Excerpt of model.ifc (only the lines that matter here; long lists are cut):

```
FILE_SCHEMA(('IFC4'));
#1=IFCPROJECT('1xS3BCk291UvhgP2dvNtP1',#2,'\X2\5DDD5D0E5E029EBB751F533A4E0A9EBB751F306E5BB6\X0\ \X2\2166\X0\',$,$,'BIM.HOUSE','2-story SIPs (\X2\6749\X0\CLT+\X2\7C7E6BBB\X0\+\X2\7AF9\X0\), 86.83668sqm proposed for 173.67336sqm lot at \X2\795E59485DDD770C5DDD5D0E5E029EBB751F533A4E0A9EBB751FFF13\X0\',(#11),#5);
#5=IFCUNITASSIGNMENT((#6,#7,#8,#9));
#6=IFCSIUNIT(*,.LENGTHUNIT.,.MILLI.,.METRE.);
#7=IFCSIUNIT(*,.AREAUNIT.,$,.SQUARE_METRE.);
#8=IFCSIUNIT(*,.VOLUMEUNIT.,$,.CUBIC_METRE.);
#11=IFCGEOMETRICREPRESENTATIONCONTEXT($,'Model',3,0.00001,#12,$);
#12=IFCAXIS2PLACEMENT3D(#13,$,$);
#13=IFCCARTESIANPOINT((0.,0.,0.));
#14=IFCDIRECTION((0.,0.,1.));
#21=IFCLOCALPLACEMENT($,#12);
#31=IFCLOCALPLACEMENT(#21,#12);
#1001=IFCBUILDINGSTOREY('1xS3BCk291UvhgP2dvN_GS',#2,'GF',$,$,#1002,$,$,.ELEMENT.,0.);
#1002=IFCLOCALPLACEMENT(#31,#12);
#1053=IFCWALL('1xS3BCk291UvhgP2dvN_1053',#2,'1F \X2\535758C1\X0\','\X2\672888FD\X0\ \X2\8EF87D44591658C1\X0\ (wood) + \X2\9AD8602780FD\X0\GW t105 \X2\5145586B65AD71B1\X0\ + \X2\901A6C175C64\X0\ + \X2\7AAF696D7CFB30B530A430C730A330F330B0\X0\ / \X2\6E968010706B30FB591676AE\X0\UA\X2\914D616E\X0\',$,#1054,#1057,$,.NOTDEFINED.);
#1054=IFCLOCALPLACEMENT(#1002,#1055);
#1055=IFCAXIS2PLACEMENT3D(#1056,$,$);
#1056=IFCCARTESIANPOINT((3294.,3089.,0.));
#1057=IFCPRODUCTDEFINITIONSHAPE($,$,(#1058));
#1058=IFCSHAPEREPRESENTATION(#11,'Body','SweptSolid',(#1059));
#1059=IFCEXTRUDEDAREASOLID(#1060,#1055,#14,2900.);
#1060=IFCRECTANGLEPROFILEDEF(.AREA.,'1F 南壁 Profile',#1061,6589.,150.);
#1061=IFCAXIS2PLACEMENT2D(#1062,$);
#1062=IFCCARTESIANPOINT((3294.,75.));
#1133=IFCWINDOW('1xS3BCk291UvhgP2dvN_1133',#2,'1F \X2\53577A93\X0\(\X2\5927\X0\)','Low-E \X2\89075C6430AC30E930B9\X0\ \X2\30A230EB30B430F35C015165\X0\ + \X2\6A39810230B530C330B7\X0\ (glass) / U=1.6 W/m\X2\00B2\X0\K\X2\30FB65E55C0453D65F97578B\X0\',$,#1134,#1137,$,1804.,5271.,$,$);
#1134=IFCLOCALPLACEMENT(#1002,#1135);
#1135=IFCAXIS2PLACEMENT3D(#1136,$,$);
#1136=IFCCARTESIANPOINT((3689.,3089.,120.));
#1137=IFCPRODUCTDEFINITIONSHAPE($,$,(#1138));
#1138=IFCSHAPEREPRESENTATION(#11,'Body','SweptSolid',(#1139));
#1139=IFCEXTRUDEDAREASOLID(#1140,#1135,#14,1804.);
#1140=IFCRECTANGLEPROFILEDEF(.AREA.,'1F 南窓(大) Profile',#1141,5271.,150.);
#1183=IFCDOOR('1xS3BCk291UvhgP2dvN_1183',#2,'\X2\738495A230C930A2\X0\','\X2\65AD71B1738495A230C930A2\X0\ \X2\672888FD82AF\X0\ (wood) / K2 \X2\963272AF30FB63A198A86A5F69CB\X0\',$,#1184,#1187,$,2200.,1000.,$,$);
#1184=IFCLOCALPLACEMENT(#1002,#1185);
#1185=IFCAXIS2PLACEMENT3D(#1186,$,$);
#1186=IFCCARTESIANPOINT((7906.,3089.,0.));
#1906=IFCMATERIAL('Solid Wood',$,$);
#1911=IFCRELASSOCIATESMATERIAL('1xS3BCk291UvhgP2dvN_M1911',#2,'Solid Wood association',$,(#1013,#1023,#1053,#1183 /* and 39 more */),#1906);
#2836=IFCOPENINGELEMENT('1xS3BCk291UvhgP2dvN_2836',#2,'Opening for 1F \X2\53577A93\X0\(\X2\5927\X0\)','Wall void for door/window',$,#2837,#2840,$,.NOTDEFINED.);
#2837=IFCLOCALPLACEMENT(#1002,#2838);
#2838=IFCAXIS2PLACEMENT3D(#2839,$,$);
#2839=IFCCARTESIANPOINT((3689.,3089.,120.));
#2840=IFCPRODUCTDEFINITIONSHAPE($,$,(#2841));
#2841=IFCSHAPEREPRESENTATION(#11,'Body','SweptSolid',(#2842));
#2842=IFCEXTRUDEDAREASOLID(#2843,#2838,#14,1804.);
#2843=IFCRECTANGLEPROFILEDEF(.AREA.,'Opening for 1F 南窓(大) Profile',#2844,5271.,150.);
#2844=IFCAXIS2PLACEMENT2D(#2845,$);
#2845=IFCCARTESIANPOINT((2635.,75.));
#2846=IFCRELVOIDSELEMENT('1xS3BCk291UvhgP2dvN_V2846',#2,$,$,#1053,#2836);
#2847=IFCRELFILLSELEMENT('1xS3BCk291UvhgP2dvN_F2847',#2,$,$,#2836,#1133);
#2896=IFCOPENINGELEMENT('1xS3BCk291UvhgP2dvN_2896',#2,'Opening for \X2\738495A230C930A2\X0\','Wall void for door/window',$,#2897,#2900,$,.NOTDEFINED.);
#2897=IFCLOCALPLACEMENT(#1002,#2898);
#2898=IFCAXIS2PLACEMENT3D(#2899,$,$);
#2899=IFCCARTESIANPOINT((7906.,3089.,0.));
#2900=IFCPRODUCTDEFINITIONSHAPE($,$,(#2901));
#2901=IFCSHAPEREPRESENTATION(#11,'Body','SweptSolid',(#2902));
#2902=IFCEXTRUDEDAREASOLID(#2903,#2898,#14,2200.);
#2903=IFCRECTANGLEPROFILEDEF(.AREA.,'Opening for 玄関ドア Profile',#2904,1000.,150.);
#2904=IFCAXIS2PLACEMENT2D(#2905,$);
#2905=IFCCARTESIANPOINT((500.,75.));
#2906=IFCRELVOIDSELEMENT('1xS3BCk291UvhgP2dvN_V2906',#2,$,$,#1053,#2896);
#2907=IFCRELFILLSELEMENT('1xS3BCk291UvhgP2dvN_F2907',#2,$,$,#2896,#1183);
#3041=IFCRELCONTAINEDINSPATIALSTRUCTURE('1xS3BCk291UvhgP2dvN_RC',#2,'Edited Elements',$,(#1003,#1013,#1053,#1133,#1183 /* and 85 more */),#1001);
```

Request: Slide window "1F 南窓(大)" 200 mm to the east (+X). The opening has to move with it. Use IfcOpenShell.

```python
import ifcopenshell
import ifcopenshell.api.geometry
import ifcopenshell.util.placement
import ifcopenshell.util.unit

model = ifcopenshell.open("model.ifc")
unit_scale = ifcopenshell.util.unit.calculate_unit_scale(model)

window = model.by_guid("1xS3BCk291UvhgP2dvN_1133")
opening = window.FillsVoids[0].RelatingOpeningElement
wall = opening.VoidsElements[0].RelatingBuildingElement

wall_matrix = ifcopenshell.util.placement.get_local_placement(wall.ObjectPlacement)
shift = wall_matrix[:3, 0] * 0.2 / unit_scale
before = ifcopenshell.util.placement.get_local_placement(window.ObjectPlacement)[:3, 3].copy()

# The window is not placed relative to its opening, so move both.
for product in (opening, window):
    matrix = ifcopenshell.util.placement.get_local_placement(product.ObjectPlacement)
    matrix[:3, 3] += shift
    ifcopenshell.api.geometry.edit_object_placement(model, product=product, matrix=matrix, is_si=False)

after = ifcopenshell.util.placement.get_local_placement(window.ObjectPlacement)[:3, 3]
print("window moved by", (after - before).round(3) + 0.0)

model.write("model_edited.ifc")
```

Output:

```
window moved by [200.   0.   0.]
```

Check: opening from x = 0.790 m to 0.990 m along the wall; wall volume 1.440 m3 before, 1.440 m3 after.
